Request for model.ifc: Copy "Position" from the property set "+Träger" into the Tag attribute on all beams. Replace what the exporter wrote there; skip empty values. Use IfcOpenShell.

First a look at what the model holds.

```python
import ifcopenshell
import ifcopenshell.util.element

model = ifcopenshell.open("model.ifc")
print(model.schema)
beams = model.by_type("IfcBeam")
print(len(beams), "beams")
for e in beams[:8]:
    source = ifcopenshell.util.element.get_pset(e, "+Träger", "Position")
    target = e.Tag
    print(e.id(), repr(source), repr(target), sep=" | ")
```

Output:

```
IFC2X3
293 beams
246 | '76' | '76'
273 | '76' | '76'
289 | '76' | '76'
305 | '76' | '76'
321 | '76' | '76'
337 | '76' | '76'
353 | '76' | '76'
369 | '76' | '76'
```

```python
import ifcopenshell
import ifcopenshell.util.element

model = ifcopenshell.open("model.ifc")

count = 0
for e in model.by_type("IfcBeam"):
    value = ifcopenshell.util.element.get_pset(e, "+Träger", "Position")
    current = e.Tag
    if not value or not value.strip() or current == value:
        continue
    e.Tag = value
    count += 1

print(count, "beams updated")

model.write("model_updated.ifc")
```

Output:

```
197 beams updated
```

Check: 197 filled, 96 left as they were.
